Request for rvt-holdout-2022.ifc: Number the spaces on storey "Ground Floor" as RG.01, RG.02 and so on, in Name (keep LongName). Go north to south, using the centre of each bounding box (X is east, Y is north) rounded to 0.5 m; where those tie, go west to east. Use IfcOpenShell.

First a look at what the model holds.

```python
import ifcopenshell
import ifcopenshell.util.element
import ifcopenshell.util.placement

model = ifcopenshell.open("rvt-holdout-2022.ifc")
print(model.schema)
storey = next(s for s in model.by_type("IfcBuildingStorey") if s.Name == "Ground Floor")
spaces = [e for e in ifcopenshell.util.element.get_decomposition(storey) if e.is_a("IfcSpace")]
for e in sorted(spaces, key=lambda e: e.id()):
    origin = ifcopenshell.util.placement.get_local_placement(e.ObjectPlacement)[:3, 3]
    print(e.id(), e.Name, e.LongName, origin.round(2) + 0.0, sep=" | ")
```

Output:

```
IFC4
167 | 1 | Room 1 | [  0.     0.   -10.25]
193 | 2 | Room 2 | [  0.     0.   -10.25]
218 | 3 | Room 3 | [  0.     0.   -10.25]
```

```python
import ifcopenshell
import ifcopenshell.geom
import ifcopenshell.util.element
import ifcopenshell.util.shape

model = ifcopenshell.open("rvt-holdout-2022.ifc")
settings = ifcopenshell.geom.settings()
settings.set("use-world-coords", True)


def centre(element):
    shape = ifcopenshell.geom.create_shape(settings, element)
    return ifcopenshell.util.shape.get_bbox_centroid(shape.geometry)


storey = next(s for s in model.by_type("IfcBuildingStorey") if s.Name == "Ground Floor")
spaces = [e for e in ifcopenshell.util.element.get_decomposition(storey) if e.is_a("IfcSpace")]

# Insertion points can sit at a corner or the storey origin, so sort by the geometry (in metres).
centres = {e: centre(e) for e in spaces}
spaces.sort(key=lambda e: (-round(centres[e][1] / 0.5), centres[e][0]))

for i, e in enumerate(spaces, start=1):
    number = f"RG.{i:02d}"
    e.Name = number
    print(e.id(), number)

model.write("rvt-holdout-2022_v2.ifc")
```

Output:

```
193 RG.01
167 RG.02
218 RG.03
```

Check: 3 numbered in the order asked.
